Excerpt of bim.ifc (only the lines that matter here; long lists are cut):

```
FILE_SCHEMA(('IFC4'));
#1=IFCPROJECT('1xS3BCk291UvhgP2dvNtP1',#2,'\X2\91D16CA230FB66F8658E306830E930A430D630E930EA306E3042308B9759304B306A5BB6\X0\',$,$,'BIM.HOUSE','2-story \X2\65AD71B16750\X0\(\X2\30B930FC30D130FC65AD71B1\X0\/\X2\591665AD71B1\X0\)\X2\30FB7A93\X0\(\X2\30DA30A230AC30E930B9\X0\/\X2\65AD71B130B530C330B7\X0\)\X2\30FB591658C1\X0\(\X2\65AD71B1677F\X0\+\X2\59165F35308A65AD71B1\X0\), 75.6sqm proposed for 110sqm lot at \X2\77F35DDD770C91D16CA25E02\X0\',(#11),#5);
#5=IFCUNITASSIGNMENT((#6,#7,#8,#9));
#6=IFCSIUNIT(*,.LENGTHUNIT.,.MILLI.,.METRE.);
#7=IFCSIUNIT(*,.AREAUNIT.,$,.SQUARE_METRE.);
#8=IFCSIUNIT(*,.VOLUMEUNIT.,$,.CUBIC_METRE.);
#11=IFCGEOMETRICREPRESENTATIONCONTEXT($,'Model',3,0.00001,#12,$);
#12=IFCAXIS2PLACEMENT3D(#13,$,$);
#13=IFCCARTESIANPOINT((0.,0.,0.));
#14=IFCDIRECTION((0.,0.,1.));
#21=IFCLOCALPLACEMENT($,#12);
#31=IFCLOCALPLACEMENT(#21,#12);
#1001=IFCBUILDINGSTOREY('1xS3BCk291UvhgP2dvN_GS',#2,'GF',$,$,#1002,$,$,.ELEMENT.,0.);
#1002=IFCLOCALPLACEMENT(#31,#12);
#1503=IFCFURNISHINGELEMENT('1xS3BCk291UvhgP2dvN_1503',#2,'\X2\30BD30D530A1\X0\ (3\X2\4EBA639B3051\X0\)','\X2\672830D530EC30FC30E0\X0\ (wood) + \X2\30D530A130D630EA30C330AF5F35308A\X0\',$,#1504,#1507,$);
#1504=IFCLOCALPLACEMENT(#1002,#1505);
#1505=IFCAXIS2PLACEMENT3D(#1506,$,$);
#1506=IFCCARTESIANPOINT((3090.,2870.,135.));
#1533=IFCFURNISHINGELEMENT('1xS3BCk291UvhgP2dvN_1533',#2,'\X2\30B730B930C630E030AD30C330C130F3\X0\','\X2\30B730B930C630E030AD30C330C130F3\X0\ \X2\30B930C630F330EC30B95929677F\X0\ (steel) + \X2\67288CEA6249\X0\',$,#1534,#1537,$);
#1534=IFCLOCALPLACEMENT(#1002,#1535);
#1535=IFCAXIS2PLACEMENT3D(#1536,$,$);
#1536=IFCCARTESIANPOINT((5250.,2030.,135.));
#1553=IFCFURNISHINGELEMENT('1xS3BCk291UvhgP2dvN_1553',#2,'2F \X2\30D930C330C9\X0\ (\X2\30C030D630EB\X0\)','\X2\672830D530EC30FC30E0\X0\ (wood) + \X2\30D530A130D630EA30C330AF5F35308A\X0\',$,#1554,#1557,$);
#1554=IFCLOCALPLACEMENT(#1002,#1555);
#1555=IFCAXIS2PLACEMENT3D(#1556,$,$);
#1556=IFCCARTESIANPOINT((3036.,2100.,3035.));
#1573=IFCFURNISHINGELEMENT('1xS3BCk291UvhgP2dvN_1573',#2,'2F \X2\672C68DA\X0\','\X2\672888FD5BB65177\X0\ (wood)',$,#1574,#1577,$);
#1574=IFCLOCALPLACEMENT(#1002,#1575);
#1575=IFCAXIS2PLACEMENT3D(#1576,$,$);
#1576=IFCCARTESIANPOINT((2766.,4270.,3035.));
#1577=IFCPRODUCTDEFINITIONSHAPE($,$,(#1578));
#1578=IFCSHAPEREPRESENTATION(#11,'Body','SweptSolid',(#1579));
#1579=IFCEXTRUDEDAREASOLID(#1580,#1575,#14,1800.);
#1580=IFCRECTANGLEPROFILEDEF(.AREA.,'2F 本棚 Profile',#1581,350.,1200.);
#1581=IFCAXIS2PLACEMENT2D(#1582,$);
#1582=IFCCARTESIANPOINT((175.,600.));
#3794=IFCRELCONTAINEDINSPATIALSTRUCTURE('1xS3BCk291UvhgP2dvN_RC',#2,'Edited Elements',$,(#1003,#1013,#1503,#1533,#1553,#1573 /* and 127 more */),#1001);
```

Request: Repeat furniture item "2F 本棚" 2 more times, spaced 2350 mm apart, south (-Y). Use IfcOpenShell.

```python
import numpy as np
import ifcopenshell
import ifcopenshell.api.geometry
import ifcopenshell.api.root
import ifcopenshell.util.element
import ifcopenshell.util.placement
import ifcopenshell.util.unit

model = ifcopenshell.open("bim.ifc")
unit_scale = ifcopenshell.util.unit.calculate_unit_scale(model)


def reuse_history(source, copy):
    """copy_class also copies each property set's owner history, people and application; keep the originals."""
    for rel in copy.IsDefinedBy:
        if rel.is_a("IfcRelDefinesByProperties") and (history := rel.RelatingPropertyDefinition.OwnerHistory):
            rel.RelatingPropertyDefinition.OwnerHistory = source.OwnerHistory
            ifcopenshell.util.element.remove_deep2(model, history)


source = model.by_guid("1xS3BCk291UvhgP2dvN_1573")
base = ifcopenshell.util.placement.get_local_placement(source.ObjectPlacement)
step = np.array([0.0, -1.0, 0.0]) * 2.35 / unit_scale

for i in range(1, 3):
    copy = ifcopenshell.api.root.copy_class(model, product=source)
    copy.Representation = ifcopenshell.util.element.copy_deep(
        model, source.Representation, exclude=["IfcGeometricRepresentationContext", "IfcRepresentationMap"]
    )
    reuse_history(source, copy)
    matrix = base.copy()
    matrix[:3, 3] += i * step
    print("added at", matrix[:3, 3].round(3) + 0.0)
    ifcopenshell.api.geometry.edit_object_placement(model, product=copy, matrix=matrix, is_si=False)

model.write("bim_v2.ifc")
```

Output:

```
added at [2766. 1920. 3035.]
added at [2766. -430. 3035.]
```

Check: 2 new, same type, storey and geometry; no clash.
